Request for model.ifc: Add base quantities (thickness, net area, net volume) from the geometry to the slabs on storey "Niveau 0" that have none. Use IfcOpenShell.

First a look at what the model holds.

```python
import ifcopenshell
import ifcopenshell.util.element
import ifcopenshell.util.unit

model = ifcopenshell.open("model.ifc")
print(model.schema)
for unit_type in ("LENGTHUNIT", "AREAUNIT", "VOLUMEUNIT"):
    print(unit_type, ifcopenshell.util.unit.calculate_unit_scale(model, unit_type))
storey = next(s for s in model.by_type("IfcBuildingStorey") if s.Name == "Niveau 0")
slabs = [e for e in ifcopenshell.util.element.get_decomposition(storey) if e.is_a("IfcSlab")]
for e in sorted(slabs, key=lambda e: e.id()):
    print(e.id(), e.is_a(), e.Name, list(ifcopenshell.util.element.get_psets(e, qtos_only=True)), sep=" | ")
```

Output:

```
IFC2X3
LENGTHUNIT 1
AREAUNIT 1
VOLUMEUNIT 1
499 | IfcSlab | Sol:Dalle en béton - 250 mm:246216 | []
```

```python
import ifcopenshell
import ifcopenshell.api.pset
import ifcopenshell.geom
import ifcopenshell.util.element
import ifcopenshell.util.shape
import ifcopenshell.util.unit

model = ifcopenshell.open("model.ifc")
unit_scale = ifcopenshell.util.unit.calculate_unit_scale(model)
area_scale = ifcopenshell.util.unit.calculate_unit_scale(model, "AREAUNIT")
volume_scale = ifcopenshell.util.unit.calculate_unit_scale(model, "VOLUMEUNIT")
settings = ifcopenshell.geom.settings()

storey = next(s for s in model.by_type("IfcBuildingStorey") if s.Name == "Niveau 0")
slabs = [e for e in ifcopenshell.util.element.get_decomposition(storey) if e.is_a("IfcSlab")]

for e in sorted(slabs, key=lambda e: e.id()):
    if ifcopenshell.util.element.get_psets(e, qtos_only=True, should_inherit=False):
        continue
    # Geometry comes back in metres, in the element's own axes.
    shape = ifcopenshell.geom.create_shape(settings, e)
    values = {
        "Width": ifcopenshell.util.shape.get_z(shape.geometry) / unit_scale,
        "NetArea": ifcopenshell.util.shape.get_footprint_area(shape.geometry) / area_scale,
        "NetVolume": ifcopenshell.util.shape.get_volume(shape.geometry) / volume_scale,
    }
    qto = ifcopenshell.api.pset.add_qto(model, product=e, name="BaseQuantities")
    ifcopenshell.api.pset.edit_qto(model, qto=qto, properties=values)
    print(e.id(), {k: round(v, 3) for k, v in values.items()})

model.write("model_v2.ifc")
```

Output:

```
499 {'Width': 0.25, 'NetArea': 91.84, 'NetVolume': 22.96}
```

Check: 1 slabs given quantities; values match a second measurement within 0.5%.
